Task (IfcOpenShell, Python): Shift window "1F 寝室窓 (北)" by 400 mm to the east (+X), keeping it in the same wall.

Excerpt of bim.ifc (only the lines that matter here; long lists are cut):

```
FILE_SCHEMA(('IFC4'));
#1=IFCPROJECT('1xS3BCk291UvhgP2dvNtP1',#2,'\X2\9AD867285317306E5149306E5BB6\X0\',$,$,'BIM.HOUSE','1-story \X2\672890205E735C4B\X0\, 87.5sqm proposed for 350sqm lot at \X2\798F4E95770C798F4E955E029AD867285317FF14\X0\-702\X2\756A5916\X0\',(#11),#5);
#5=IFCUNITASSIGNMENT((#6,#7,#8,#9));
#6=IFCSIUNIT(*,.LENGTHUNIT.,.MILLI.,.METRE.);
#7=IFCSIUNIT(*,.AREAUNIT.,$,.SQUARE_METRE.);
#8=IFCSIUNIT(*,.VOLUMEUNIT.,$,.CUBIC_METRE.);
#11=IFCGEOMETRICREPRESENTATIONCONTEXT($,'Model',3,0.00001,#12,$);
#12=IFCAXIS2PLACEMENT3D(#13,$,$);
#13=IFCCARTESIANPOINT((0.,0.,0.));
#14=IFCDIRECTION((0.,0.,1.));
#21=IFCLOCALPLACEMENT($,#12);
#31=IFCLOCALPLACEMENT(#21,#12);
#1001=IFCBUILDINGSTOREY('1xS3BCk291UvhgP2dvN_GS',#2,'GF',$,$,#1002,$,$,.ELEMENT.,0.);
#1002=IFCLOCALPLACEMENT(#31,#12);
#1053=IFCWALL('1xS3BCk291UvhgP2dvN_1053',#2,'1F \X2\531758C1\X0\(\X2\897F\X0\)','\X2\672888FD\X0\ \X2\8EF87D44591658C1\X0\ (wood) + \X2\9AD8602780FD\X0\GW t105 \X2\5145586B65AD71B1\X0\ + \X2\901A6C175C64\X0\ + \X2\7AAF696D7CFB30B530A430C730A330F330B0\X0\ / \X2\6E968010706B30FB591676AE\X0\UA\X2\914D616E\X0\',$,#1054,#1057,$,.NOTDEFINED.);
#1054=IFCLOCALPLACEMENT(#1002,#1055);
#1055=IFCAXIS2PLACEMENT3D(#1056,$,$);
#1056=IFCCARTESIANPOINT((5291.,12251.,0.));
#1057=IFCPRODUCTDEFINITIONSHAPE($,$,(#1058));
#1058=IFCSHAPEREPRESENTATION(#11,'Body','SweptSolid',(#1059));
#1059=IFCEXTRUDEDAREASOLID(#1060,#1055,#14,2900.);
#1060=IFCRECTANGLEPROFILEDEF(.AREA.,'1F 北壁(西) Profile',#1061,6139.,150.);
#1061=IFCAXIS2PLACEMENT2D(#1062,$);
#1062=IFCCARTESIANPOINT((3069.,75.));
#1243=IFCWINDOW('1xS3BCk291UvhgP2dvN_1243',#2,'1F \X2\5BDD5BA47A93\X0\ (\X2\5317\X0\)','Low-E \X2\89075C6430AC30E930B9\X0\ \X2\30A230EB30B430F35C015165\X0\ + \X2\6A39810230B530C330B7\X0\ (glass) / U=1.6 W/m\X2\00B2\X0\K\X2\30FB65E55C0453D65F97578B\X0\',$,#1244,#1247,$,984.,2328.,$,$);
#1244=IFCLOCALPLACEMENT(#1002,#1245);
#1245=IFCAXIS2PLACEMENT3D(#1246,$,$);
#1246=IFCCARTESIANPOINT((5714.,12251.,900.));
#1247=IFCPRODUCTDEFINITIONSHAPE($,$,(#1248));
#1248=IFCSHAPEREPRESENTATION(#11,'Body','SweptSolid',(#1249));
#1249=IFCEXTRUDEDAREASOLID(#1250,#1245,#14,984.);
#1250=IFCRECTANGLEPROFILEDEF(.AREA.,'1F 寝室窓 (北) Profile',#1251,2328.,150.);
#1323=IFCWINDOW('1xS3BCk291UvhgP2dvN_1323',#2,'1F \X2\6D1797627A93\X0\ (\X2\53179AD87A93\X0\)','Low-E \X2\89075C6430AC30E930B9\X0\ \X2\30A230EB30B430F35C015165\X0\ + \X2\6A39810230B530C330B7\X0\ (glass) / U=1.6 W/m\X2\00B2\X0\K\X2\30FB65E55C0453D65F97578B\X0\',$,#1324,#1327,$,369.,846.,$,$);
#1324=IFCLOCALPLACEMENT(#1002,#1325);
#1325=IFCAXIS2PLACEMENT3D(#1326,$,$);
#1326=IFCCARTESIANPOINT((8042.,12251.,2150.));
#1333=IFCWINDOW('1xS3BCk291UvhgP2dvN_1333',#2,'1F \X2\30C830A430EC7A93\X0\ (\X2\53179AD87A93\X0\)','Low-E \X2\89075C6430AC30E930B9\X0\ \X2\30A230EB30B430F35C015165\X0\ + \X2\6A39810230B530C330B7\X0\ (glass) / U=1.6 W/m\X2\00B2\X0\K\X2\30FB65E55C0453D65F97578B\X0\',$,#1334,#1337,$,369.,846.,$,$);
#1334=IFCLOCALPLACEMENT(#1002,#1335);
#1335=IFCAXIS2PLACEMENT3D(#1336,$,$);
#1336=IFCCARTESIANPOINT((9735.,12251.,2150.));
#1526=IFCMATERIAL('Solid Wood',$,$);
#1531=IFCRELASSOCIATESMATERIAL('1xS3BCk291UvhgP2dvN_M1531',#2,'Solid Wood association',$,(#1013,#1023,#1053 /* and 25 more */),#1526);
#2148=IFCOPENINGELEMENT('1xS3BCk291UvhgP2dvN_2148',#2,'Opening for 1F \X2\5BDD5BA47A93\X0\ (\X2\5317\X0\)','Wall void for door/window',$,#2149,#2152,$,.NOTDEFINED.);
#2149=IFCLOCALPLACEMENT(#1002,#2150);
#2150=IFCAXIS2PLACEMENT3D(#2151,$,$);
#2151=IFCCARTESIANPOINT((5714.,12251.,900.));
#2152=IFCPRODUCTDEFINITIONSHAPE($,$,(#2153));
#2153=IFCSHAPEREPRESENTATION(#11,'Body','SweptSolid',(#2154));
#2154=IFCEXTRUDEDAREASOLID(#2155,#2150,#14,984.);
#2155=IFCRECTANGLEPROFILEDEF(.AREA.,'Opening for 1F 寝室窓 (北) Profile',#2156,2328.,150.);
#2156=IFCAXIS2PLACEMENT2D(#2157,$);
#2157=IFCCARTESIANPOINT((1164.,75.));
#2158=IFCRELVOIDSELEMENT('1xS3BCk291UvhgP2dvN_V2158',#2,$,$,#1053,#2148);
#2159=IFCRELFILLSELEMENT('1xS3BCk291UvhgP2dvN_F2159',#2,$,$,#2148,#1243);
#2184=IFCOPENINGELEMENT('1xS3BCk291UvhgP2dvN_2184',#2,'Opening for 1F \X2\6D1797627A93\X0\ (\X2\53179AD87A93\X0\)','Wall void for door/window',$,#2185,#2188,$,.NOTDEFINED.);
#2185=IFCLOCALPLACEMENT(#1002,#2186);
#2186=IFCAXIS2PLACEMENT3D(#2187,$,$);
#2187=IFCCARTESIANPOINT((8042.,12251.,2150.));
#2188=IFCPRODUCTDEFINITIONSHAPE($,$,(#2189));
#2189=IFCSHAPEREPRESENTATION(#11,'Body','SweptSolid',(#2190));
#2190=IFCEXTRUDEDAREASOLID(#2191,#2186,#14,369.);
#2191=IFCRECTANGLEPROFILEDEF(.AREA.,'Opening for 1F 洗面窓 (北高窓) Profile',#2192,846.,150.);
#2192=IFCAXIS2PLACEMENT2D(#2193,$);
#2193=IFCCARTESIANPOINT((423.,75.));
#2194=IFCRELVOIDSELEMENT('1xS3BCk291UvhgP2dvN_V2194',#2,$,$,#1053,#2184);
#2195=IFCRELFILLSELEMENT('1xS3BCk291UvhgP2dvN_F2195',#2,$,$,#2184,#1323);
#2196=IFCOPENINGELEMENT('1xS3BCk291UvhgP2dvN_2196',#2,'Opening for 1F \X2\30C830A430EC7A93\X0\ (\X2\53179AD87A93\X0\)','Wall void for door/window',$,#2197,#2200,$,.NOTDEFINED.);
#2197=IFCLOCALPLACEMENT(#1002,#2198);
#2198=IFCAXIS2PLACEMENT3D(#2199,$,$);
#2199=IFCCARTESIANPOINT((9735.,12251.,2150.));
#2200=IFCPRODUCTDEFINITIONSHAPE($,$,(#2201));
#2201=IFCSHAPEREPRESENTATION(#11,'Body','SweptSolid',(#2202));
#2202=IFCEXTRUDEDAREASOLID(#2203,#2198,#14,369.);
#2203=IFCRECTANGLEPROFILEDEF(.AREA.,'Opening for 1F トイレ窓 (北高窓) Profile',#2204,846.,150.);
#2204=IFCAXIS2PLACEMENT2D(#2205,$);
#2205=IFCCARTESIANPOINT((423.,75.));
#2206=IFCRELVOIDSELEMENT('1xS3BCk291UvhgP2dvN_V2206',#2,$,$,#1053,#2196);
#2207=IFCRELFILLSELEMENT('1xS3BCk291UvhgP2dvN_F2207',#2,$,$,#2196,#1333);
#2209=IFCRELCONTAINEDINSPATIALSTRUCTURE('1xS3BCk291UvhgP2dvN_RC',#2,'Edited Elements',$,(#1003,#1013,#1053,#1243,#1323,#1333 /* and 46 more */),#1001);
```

```python
import ifcopenshell
import ifcopenshell.api.geometry
import ifcopenshell.util.placement
import ifcopenshell.util.unit

model = ifcopenshell.open("bim.ifc")
unit_scale = ifcopenshell.util.unit.calculate_unit_scale(model)

window = model.by_guid("1xS3BCk291UvhgP2dvN_1243")
opening = window.FillsVoids[0].RelatingOpeningElement
wall = opening.VoidsElements[0].RelatingBuildingElement

wall_matrix = ifcopenshell.util.placement.get_local_placement(wall.ObjectPlacement)
shift = wall_matrix[:3, 0] * 0.4 / unit_scale
before = ifcopenshell.util.placement.get_local_placement(window.ObjectPlacement)[:3, 3].copy()

# The window is not placed relative to its opening, so move both.
for product in (opening, window):
    matrix = ifcopenshell.util.placement.get_local_placement(product.ObjectPlacement)
    matrix[:3, 3] += shift
    ifcopenshell.api.geometry.edit_object_placement(model, product=product, matrix=matrix, is_si=False)

after = ifcopenshell.util.placement.get_local_placement(window.ObjectPlacement)[:3, 3]
print("window moved by", (after - before).round(3) + 0.0)

model.write("bim_v2.ifc")
```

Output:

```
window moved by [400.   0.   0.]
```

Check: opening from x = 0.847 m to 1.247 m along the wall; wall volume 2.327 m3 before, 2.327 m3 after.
